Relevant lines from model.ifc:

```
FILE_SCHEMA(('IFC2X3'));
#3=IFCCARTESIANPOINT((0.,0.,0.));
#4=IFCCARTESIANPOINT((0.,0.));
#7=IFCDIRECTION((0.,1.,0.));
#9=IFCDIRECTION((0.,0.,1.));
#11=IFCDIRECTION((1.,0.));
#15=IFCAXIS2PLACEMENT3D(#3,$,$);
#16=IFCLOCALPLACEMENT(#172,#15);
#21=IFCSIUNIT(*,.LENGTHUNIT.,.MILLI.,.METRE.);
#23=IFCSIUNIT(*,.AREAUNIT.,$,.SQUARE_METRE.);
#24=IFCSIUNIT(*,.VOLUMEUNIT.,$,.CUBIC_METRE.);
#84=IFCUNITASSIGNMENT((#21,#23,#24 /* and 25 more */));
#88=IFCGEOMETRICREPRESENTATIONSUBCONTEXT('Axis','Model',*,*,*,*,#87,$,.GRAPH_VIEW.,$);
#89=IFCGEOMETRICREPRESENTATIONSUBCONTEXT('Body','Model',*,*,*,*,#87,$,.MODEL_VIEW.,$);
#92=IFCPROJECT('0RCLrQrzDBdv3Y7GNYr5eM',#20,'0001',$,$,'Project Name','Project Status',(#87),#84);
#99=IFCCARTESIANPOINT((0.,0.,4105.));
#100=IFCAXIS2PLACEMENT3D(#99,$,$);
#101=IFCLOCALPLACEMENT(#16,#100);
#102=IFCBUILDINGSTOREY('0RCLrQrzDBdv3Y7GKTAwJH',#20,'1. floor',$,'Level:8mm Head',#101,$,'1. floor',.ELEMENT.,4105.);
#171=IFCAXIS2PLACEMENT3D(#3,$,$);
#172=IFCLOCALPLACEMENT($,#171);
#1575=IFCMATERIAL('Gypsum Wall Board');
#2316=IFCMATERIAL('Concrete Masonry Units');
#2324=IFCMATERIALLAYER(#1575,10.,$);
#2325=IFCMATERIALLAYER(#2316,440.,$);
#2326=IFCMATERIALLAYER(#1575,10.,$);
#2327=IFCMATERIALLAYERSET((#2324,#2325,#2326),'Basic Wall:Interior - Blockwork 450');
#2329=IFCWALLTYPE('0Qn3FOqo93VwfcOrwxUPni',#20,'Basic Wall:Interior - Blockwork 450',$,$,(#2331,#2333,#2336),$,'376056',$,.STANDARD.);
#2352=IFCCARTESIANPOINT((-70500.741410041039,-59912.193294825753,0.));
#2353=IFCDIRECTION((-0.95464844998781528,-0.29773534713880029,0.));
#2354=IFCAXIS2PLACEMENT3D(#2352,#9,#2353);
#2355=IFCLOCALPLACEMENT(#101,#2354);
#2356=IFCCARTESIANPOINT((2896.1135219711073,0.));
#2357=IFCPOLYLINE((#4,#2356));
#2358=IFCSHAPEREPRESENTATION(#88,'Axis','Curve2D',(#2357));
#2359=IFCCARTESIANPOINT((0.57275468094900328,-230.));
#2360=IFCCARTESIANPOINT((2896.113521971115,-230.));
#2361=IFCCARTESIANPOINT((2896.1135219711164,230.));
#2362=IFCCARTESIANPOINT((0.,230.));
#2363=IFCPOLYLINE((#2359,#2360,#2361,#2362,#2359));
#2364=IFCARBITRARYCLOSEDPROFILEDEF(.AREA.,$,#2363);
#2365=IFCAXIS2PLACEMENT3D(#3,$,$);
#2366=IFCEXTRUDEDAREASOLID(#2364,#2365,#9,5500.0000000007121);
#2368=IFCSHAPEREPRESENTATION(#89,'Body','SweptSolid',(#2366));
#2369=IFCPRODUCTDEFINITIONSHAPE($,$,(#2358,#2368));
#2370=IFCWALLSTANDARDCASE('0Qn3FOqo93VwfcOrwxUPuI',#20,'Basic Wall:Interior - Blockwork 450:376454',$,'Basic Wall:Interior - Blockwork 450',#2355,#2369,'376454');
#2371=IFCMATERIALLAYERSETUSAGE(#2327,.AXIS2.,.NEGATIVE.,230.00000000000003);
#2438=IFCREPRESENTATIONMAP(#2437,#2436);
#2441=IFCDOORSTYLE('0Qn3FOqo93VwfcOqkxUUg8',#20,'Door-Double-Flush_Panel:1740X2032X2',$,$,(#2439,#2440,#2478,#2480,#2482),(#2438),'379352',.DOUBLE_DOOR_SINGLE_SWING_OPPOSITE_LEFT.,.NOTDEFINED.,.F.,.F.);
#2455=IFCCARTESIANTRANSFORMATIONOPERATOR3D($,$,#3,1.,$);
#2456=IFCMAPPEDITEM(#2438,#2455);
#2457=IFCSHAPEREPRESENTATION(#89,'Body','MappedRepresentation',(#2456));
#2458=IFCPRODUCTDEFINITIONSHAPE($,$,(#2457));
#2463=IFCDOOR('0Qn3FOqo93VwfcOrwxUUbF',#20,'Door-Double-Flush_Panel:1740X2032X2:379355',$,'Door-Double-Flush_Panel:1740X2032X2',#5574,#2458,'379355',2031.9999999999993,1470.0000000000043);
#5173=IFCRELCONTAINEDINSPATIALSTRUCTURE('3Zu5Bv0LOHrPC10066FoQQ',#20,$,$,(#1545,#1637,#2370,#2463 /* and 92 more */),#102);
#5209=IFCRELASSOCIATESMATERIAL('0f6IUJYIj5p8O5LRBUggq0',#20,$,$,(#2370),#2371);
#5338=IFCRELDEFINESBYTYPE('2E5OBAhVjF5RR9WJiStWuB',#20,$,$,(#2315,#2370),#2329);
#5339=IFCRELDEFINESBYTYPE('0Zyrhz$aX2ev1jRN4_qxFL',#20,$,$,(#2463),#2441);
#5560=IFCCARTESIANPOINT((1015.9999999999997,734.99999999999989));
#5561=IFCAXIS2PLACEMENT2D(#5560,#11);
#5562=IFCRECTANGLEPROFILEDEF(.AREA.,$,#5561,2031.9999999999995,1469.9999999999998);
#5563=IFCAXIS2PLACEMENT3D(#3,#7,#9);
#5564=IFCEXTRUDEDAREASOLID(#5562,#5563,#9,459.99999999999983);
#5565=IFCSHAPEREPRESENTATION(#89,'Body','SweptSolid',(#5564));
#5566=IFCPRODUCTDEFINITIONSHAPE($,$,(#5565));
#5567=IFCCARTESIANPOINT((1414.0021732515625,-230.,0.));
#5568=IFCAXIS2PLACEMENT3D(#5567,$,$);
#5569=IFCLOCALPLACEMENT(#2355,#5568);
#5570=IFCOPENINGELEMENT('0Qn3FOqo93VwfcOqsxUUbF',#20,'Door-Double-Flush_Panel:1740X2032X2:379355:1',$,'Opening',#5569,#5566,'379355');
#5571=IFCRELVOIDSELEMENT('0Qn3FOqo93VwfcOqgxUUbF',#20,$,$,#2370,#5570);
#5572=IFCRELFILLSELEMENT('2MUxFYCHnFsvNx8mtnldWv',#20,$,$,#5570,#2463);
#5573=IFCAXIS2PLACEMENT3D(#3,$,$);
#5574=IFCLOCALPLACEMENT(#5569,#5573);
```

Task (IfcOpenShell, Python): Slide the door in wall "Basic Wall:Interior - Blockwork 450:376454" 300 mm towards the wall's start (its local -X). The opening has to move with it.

```python
import ifcopenshell
import ifcopenshell.api.geometry
import ifcopenshell.util.placement
import ifcopenshell.util.unit

model = ifcopenshell.open("model.ifc")
unit_scale = ifcopenshell.util.unit.calculate_unit_scale(model)

door = model.by_guid("0Qn3FOqo93VwfcOrwxUUbF")
opening = door.FillsVoids[0].RelatingOpeningElement
wall = opening.VoidsElements[0].RelatingBuildingElement

wall_matrix = ifcopenshell.util.placement.get_local_placement(wall.ObjectPlacement)
shift = wall_matrix[:3, 0] * -0.3 / unit_scale
before = ifcopenshell.util.placement.get_local_placement(door.ObjectPlacement)[:3, 3].copy()

# The door is placed relative to its opening, so it follows when the opening moves.
matrix = ifcopenshell.util.placement.get_local_placement(opening.ObjectPlacement)
matrix[:3, 3] += shift
ifcopenshell.api.geometry.edit_object_placement(
    model, product=opening, matrix=matrix, is_si=False, should_transform_children=True
)

after = ifcopenshell.util.placement.get_local_placement(door.ObjectPlacement)[:3, 3]
print("door moved by", (after - before).round(3) + 0.0)

model.write("model-out.ifc")
```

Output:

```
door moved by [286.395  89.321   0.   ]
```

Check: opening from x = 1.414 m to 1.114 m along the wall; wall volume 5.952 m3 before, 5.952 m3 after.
